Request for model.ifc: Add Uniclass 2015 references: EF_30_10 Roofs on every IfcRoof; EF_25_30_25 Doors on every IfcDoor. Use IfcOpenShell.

First a look at what the model holds.

```python
import ifcopenshell

model = ifcopenshell.open("model.ifc")
print(model.schema)
print("classifications:", [c.Name for c in model.by_type("IfcClassification")])
for ifc_class in ("IfcDoor", "IfcRoof", "IfcStair", "IfcWall", "IfcWindow"):
    print(ifc_class, len(model.by_type(ifc_class)))
```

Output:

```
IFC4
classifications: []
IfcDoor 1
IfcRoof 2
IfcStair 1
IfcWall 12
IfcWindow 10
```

```python
import ifcopenshell
import ifcopenshell.api.classification

model = ifcopenshell.open("model.ifc")

system = ifcopenshell.api.classification.add_classification(model, classification="Uniclass 2015")

codes = {
    "IfcRoof": ("EF_30_10", "Roofs"),
    "IfcDoor": ("EF_25_30_25", "Doors"),
}
for ifc_class, (code, name) in codes.items():
    products = model.by_type(ifc_class)
    ifcopenshell.api.classification.add_reference(
        model, products=products, classification=system, identification=code, name=name
    )
    print(code, len(products))

model.write("model-out.ifc")
```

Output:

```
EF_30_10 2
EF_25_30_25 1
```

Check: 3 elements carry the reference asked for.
